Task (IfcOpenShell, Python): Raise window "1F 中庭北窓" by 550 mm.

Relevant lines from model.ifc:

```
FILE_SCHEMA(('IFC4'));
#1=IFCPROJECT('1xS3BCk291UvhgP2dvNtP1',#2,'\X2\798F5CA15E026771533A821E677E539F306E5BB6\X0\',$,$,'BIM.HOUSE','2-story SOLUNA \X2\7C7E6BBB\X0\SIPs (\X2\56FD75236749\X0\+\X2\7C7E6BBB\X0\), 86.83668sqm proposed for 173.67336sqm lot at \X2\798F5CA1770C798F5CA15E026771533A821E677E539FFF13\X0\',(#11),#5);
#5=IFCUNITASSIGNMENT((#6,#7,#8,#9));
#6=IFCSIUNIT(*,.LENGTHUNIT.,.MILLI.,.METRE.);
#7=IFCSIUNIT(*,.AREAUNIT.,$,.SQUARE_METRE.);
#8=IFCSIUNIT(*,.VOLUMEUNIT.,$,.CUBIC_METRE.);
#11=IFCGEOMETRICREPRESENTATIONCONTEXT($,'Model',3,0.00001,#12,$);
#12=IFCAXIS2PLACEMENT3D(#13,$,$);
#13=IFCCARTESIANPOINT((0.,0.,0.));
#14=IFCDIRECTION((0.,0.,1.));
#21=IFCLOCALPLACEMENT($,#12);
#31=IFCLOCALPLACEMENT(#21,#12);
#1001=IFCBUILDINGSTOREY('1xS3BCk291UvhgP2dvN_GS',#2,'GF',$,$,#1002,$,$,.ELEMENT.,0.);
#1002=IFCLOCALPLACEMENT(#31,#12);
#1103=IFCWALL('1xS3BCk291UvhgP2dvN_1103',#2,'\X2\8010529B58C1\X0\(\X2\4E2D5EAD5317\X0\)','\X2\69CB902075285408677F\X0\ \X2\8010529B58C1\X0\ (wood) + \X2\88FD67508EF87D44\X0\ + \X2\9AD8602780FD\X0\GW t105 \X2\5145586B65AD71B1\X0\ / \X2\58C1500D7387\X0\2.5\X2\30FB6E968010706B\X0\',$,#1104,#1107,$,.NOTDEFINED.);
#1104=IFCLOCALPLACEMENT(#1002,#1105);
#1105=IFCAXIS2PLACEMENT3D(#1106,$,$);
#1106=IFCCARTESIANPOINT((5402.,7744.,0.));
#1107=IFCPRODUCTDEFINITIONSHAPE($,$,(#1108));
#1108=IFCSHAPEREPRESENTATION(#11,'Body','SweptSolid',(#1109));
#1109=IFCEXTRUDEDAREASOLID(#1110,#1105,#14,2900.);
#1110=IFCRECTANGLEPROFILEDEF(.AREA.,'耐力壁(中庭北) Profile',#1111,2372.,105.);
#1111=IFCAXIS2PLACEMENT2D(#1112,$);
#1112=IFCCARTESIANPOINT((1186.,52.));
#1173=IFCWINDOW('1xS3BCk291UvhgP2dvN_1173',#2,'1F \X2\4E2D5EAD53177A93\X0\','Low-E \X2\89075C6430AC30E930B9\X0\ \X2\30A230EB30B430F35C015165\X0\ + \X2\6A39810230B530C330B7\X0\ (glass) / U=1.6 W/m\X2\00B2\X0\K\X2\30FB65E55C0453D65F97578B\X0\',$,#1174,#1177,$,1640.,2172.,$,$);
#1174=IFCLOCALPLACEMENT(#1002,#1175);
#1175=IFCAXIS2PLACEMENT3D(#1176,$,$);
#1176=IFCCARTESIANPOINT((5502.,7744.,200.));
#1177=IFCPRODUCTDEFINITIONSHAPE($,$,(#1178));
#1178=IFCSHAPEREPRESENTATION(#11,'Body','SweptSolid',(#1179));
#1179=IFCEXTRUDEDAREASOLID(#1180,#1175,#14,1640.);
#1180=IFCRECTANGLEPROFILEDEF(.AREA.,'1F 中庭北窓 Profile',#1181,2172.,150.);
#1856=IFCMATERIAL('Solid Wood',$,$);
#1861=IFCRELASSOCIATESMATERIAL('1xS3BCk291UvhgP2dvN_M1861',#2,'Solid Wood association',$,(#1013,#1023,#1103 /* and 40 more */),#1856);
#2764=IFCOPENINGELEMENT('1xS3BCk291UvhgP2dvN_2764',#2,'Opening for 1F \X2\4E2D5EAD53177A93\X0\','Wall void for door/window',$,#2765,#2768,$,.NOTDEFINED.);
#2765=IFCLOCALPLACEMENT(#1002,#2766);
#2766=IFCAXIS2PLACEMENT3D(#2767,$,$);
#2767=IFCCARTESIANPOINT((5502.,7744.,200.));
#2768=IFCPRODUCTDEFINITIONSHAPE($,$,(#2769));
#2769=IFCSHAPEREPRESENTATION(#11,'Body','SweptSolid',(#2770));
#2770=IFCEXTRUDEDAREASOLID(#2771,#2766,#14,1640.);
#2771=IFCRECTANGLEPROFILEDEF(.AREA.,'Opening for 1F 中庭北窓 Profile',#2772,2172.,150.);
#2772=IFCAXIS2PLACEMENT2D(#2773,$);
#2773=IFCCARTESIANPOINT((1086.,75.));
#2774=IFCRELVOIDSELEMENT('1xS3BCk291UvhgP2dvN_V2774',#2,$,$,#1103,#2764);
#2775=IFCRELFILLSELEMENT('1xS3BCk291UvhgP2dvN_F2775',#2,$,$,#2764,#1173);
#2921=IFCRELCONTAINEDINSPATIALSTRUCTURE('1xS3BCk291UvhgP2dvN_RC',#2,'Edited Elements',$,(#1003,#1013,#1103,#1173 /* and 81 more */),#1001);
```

```python
import numpy as np
import ifcopenshell
import ifcopenshell.api.geometry
import ifcopenshell.util.placement
import ifcopenshell.util.unit

model = ifcopenshell.open("model.ifc")
unit_scale = ifcopenshell.util.unit.calculate_unit_scale(model)

window = model.by_guid("1xS3BCk291UvhgP2dvN_1173")
opening = window.FillsVoids[0].RelatingOpeningElement
dz = 0.55 / unit_scale

shift = np.array([0.0, 0.0, dz])
# The window is not placed relative to its opening, so move both.
for product in (opening, window):
    matrix = ifcopenshell.util.placement.get_local_placement(product.ObjectPlacement)
    matrix[:3, 3] += shift
    ifcopenshell.api.geometry.edit_object_placement(model, product=product, matrix=matrix, is_si=False)

print(f"moved by {dz * unit_scale:+.3f} m")

model.write("model_updated.ifc")
```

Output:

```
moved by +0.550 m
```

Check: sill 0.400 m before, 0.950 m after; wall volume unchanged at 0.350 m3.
